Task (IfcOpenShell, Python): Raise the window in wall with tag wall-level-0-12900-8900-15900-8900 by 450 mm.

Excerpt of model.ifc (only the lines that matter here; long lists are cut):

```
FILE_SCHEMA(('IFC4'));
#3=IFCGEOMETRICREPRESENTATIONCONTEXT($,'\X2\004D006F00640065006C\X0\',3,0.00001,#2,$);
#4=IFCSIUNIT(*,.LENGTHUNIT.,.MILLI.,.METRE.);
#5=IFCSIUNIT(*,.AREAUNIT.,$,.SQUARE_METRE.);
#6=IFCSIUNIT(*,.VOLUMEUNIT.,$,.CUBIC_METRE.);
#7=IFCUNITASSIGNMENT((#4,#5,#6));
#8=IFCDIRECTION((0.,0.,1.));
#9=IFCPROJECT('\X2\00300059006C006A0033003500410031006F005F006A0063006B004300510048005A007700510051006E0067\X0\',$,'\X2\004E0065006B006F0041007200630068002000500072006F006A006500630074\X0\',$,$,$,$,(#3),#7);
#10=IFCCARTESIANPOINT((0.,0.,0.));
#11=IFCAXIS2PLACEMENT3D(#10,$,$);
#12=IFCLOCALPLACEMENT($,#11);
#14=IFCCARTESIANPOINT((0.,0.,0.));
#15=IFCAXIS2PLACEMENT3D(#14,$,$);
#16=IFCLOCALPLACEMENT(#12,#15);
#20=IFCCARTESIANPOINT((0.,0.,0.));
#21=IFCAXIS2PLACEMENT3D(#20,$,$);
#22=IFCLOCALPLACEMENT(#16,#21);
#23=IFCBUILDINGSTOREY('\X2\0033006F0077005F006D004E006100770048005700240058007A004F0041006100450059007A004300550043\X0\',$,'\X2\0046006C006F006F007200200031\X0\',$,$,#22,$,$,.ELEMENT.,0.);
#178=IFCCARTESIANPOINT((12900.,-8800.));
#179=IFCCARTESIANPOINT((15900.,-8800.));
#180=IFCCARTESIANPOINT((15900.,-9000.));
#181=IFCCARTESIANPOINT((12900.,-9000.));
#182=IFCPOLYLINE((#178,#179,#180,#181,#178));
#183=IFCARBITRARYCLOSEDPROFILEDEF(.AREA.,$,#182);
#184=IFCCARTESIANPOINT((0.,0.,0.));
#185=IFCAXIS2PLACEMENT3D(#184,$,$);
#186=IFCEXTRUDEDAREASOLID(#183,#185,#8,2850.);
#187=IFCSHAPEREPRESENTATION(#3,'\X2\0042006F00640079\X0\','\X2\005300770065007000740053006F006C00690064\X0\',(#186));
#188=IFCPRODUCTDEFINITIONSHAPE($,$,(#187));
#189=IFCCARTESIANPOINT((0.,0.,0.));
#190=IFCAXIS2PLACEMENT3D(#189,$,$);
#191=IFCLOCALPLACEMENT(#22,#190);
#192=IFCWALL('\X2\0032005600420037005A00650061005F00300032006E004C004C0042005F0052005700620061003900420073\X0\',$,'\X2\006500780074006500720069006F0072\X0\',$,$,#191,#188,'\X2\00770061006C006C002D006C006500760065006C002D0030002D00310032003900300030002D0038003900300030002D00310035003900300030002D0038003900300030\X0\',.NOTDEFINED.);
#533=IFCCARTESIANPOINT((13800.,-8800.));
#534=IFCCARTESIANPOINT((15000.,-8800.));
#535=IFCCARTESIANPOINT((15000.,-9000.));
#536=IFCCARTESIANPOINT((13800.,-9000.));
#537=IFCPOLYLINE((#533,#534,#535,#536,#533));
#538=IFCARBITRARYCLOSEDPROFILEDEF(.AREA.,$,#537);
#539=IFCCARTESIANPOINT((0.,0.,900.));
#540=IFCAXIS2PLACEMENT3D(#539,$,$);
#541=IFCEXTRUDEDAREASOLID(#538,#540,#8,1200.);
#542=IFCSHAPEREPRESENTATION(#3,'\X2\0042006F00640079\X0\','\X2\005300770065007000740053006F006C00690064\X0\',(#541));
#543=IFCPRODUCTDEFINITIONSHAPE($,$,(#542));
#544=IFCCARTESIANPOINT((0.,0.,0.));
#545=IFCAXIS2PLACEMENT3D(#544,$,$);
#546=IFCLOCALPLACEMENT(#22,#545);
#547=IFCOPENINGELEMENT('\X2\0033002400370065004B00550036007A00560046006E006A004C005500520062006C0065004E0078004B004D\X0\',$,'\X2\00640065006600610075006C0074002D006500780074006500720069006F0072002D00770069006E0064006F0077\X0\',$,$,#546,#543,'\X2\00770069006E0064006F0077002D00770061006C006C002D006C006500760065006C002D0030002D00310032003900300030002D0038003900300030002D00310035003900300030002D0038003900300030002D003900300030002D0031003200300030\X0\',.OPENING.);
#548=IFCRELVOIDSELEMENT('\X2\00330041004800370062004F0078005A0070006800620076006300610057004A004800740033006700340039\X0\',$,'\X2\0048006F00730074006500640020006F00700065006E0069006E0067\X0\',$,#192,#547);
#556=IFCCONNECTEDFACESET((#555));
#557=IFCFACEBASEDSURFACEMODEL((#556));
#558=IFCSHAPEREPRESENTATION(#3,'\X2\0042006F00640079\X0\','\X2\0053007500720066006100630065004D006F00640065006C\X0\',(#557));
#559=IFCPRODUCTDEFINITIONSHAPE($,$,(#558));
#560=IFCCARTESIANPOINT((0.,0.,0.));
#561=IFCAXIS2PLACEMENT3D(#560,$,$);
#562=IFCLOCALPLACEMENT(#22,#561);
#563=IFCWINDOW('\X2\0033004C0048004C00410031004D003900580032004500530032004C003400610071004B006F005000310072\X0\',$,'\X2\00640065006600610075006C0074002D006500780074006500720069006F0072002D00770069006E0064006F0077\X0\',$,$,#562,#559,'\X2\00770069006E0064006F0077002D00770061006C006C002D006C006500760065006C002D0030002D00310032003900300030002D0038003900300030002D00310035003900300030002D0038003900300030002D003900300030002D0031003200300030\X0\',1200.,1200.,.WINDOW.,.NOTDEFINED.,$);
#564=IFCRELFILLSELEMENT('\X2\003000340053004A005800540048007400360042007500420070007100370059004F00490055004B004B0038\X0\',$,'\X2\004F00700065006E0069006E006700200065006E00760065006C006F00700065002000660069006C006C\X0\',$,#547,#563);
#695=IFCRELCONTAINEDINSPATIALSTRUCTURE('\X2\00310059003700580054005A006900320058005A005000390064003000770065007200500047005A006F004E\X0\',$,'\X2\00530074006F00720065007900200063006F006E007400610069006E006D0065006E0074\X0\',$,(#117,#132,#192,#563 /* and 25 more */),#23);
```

```python
import numpy as np
import ifcopenshell
import ifcopenshell.api.geometry
import ifcopenshell.util.placement
import ifcopenshell.util.unit

model = ifcopenshell.open("model.ifc")
unit_scale = ifcopenshell.util.unit.calculate_unit_scale(model)

window = model.by_guid("3LHLA1M9X2ES2L4aqKoP1r")
opening = window.FillsVoids[0].RelatingOpeningElement
dz = 0.45 / unit_scale

shift = np.array([0.0, 0.0, dz])
# The window is not placed relative to its opening, so move both.
for product in (opening, window):
    matrix = ifcopenshell.util.placement.get_local_placement(product.ObjectPlacement)
    matrix[:3, 3] += shift
    ifcopenshell.api.geometry.edit_object_placement(model, product=product, matrix=matrix, is_si=False)

print(f"moved by {dz * unit_scale:+.3f} m")

model.write("model_v2.ifc")
```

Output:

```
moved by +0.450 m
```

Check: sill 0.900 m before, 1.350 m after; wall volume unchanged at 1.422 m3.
